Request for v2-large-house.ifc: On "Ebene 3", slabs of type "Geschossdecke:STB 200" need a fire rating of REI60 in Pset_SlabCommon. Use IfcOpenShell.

First a look at what the model holds.

```python
import ifcopenshell
import ifcopenshell.util.element

model = ifcopenshell.open("v2-large-house.ifc")
print(model.schema)
storey = next(s for s in model.by_type("IfcBuildingStorey") if s.Name == "Ebene 3")
slabs = [e for e in ifcopenshell.util.element.get_decomposition(storey) if e.is_a("IfcSlab")]
seen = {}
for e in slabs:
    element_type = ifcopenshell.util.element.get_type(e)
    key = (element_type.Name if element_type != e and element_type else None, ifcopenshell.util.element.get_pset(e, "Pset_SlabCommon", "FireRating"))
    seen[key] = seen.get(key, 0) + 1
for (name, value), count in sorted(seen.items(), key=str):
    print(count, "x", name, "|", value)
```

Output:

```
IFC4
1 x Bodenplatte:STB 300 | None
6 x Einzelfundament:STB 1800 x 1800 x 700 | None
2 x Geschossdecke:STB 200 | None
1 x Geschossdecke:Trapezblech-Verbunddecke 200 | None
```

```python
import ifcopenshell
import ifcopenshell.api.pset
import ifcopenshell.util.element

model = ifcopenshell.open("v2-large-house.ifc")

storey = next(s for s in model.by_type("IfcBuildingStorey") if s.Name == "Ebene 3")
slabs = [e for e in ifcopenshell.util.element.get_decomposition(storey) if e.is_a("IfcSlab")]

count = 0
for e in slabs:
    element_type = ifcopenshell.util.element.get_type(e)
    if element_type in (None, e) or element_type.Name != "Geschossdecke:STB 200":
        continue
    # add_pset returns the element's existing set when there is one.
    pset = ifcopenshell.api.pset.add_pset(model, product=e, name="Pset_SlabCommon")
    ifcopenshell.api.pset.edit_pset(model, pset=pset, properties={"FireRating": "REI60"})
    count += 1

print(count, "slabs updated")

model.write("v2-large-house_rev.ifc")
```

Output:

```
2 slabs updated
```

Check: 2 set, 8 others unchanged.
